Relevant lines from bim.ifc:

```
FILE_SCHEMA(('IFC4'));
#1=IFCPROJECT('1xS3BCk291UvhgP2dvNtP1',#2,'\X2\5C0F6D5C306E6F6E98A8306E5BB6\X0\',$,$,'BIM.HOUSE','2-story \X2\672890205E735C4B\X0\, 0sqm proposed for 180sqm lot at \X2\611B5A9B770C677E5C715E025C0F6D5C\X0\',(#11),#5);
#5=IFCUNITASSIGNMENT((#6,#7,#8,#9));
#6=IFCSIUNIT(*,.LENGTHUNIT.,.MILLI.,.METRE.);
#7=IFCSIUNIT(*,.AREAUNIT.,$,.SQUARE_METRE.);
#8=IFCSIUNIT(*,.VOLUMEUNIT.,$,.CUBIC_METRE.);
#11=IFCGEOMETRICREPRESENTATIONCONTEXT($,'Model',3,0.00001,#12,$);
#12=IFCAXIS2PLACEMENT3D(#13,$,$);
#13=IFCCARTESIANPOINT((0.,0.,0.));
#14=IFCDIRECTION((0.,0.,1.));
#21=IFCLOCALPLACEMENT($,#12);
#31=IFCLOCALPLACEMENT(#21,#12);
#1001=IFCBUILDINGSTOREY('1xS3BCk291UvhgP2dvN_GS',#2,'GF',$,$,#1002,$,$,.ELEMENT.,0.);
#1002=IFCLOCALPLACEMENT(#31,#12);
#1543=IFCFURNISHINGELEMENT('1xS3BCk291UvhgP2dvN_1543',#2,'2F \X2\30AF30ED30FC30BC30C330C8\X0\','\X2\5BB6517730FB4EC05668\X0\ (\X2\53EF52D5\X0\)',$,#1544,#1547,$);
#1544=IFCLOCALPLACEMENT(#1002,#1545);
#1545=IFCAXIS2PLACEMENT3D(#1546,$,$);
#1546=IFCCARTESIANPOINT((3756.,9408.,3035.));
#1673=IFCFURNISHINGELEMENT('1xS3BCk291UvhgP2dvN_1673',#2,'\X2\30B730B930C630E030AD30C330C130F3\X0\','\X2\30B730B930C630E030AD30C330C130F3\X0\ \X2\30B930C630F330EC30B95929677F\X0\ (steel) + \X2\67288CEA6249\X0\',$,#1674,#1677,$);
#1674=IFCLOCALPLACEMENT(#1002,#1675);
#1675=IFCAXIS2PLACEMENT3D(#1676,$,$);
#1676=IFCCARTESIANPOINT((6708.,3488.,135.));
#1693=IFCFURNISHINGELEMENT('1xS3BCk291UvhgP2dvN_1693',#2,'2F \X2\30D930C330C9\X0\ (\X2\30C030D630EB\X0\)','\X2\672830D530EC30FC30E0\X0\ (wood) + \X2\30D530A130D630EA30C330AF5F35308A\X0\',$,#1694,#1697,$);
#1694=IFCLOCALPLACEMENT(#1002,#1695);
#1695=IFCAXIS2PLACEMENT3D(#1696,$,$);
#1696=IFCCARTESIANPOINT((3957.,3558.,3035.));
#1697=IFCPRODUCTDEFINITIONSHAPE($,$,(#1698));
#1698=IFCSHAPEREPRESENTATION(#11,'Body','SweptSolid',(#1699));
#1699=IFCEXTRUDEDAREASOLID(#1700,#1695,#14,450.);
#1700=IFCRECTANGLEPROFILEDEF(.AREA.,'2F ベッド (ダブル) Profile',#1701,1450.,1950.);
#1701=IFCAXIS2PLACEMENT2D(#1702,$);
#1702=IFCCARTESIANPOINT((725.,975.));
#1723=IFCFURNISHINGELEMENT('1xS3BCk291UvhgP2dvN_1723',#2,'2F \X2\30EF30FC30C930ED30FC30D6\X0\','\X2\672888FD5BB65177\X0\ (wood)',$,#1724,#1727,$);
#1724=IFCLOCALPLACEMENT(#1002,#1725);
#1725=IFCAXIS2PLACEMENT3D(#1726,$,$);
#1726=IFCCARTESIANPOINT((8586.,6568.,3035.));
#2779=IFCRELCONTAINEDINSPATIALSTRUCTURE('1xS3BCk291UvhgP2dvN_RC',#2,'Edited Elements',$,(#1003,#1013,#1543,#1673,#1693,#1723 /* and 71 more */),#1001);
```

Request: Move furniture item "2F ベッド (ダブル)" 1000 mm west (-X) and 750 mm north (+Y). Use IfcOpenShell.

```python
import ifcopenshell
import ifcopenshell.api.geometry
import ifcopenshell.util.placement
import ifcopenshell.util.unit

model = ifcopenshell.open("bim.ifc")
unit_scale = ifcopenshell.util.unit.calculate_unit_scale(model)

item = model.by_guid("1xS3BCk291UvhgP2dvN_1693")
matrix = ifcopenshell.util.placement.get_local_placement(item.ObjectPlacement)
matrix[0, 3] -= 1 / unit_scale
matrix[1, 3] += 0.75 / unit_scale
ifcopenshell.api.geometry.edit_object_placement(model, product=item, matrix=matrix, is_si=False)

print(ifcopenshell.util.placement.get_local_placement(item.ObjectPlacement).round(3) + 0.0)

model.write("bim_v2.ifc")
```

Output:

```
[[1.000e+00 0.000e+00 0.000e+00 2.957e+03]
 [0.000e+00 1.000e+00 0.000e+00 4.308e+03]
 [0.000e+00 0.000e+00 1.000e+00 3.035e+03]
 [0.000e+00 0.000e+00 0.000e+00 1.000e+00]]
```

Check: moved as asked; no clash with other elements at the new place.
